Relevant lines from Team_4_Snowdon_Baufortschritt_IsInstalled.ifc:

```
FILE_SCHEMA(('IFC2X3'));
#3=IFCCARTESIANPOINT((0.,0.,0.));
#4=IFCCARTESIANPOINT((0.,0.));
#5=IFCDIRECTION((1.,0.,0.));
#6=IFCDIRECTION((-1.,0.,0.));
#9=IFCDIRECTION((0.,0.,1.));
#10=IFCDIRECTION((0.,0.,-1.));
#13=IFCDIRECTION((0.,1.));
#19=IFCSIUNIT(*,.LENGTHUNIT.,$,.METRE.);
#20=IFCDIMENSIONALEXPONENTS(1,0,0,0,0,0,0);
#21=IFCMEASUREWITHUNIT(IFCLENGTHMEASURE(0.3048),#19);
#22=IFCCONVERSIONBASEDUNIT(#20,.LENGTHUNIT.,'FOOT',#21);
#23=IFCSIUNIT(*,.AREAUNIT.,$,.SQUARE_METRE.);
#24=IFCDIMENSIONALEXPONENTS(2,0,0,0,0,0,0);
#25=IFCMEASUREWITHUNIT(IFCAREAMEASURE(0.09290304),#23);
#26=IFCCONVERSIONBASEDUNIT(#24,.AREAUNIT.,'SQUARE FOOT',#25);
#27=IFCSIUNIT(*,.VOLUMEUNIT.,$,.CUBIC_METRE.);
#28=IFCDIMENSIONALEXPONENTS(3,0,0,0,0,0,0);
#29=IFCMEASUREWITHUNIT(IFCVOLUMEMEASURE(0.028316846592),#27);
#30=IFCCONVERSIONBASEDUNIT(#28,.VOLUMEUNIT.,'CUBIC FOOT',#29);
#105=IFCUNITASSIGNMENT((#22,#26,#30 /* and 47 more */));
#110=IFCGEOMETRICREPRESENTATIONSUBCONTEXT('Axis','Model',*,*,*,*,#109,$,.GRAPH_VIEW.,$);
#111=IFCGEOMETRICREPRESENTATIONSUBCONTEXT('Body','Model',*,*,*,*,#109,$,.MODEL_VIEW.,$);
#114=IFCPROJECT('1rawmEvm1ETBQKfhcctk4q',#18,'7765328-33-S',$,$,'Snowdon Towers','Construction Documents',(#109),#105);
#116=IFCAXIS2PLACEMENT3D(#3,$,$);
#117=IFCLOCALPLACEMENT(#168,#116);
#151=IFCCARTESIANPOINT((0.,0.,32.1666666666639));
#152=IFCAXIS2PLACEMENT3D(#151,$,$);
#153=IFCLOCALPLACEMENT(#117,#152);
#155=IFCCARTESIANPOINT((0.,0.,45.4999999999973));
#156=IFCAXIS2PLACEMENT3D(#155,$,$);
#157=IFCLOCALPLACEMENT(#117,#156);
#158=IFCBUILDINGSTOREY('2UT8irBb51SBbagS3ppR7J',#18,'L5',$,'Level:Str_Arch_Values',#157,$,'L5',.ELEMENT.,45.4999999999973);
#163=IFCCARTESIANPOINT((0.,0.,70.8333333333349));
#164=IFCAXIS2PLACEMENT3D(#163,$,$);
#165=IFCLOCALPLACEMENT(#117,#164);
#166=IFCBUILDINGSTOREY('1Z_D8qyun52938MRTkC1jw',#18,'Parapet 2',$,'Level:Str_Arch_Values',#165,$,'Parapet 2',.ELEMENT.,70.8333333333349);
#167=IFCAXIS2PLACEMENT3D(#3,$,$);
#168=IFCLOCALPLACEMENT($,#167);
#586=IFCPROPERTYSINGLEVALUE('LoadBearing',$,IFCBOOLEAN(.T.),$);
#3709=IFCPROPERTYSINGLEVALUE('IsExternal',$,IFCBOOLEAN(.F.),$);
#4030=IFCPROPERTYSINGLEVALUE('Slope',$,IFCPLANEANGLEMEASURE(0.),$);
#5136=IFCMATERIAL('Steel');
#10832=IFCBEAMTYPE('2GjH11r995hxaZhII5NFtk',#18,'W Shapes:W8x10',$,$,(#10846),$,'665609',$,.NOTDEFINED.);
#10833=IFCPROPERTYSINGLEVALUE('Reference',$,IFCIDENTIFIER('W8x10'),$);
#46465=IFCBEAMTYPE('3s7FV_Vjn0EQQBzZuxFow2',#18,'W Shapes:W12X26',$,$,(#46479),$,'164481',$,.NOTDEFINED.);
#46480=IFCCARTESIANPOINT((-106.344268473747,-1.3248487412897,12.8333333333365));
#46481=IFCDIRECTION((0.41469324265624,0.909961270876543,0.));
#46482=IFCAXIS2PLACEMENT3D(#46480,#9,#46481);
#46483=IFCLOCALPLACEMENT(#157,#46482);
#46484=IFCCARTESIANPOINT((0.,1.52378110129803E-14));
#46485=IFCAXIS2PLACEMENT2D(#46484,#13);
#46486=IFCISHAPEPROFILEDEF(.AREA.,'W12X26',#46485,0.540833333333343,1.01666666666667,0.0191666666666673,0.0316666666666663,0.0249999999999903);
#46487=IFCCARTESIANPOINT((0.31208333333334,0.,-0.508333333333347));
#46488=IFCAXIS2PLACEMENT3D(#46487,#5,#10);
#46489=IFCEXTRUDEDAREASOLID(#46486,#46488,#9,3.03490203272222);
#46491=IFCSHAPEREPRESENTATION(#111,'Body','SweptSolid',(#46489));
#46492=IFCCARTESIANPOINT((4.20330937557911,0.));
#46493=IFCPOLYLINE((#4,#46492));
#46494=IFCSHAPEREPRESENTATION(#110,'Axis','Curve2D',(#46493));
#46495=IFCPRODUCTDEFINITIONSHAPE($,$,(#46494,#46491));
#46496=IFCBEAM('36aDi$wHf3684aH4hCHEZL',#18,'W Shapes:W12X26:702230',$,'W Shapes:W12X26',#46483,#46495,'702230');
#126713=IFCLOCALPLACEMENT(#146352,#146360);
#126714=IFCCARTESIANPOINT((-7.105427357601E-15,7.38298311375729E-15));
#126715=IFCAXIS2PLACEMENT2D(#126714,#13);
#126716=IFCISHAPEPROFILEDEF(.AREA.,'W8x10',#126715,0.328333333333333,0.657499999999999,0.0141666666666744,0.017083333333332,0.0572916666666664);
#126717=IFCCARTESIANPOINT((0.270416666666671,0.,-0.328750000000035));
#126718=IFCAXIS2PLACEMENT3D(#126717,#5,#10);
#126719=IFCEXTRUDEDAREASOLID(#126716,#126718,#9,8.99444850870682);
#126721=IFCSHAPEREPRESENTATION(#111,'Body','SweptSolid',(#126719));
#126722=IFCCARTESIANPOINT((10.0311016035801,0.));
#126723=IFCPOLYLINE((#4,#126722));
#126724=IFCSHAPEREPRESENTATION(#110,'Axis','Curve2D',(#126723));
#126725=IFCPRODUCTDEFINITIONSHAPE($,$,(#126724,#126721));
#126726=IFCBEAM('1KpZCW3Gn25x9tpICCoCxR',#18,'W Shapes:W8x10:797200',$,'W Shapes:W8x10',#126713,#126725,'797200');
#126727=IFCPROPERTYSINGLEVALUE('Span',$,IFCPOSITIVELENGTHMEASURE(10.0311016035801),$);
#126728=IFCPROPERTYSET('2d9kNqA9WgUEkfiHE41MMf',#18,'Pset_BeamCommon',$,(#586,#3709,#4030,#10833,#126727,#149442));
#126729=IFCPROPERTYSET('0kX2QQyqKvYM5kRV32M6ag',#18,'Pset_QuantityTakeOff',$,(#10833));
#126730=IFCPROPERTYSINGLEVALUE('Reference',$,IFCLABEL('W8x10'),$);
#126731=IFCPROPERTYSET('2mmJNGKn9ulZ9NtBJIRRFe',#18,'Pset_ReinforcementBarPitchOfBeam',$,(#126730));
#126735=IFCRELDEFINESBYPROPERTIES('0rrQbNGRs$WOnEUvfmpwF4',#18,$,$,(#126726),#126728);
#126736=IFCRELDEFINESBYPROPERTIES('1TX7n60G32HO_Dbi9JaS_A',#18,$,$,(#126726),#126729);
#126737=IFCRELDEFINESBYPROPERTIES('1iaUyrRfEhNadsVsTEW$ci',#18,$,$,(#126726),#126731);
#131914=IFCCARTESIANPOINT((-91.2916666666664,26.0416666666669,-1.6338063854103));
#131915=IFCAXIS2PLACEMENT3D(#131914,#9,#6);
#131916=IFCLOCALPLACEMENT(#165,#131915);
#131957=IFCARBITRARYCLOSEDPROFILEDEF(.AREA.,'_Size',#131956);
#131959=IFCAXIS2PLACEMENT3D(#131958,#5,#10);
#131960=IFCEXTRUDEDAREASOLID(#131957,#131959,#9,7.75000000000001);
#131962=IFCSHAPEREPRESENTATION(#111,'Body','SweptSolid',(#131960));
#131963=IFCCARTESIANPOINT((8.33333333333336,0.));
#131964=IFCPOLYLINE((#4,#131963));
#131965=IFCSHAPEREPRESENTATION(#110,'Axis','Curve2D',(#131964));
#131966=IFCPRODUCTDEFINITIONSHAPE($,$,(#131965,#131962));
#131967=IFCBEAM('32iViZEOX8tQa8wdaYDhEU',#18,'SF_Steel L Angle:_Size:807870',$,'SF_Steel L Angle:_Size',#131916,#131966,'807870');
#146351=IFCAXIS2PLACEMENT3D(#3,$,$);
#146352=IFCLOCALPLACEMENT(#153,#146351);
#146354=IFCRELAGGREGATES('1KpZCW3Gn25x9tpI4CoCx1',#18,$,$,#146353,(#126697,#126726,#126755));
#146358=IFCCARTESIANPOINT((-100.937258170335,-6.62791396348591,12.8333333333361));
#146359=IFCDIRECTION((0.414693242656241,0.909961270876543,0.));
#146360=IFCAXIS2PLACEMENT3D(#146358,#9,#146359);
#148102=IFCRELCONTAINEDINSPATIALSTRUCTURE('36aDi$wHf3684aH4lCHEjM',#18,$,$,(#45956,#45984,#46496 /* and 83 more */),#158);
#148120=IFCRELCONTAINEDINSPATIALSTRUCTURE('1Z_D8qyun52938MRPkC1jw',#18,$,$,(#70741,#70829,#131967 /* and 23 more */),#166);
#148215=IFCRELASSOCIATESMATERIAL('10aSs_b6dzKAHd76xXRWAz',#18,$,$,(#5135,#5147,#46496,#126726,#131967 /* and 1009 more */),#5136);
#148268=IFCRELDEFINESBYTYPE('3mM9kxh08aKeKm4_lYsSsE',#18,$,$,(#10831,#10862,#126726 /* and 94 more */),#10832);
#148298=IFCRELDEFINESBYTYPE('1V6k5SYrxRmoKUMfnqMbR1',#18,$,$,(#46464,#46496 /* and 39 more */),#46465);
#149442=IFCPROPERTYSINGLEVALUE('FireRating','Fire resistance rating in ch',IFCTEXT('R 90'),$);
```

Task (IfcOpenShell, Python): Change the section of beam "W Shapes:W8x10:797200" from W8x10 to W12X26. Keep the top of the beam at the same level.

```python
import ifcopenshell
import ifcopenshell.api.pset
import ifcopenshell.api.type
import ifcopenshell.util.element
import ifcopenshell.util.representation

model = ifcopenshell.open("Team_4_Snowdon_Baufortschritt_IsInstalled.ifc")

member = model.by_id(126726)
source = next(p for p in model.by_type("IfcIShapeProfileDef") if p.ProfileName == "W12X26")

body = ifcopenshell.util.representation.get_representation(member, "Model", "Body")
solid = body.Items[0]
old_profile = solid.SweptArea

# Copy the section's sizes but keep this member's own profile position.
profile = ifcopenshell.util.element.copy(model, source)
# Profiles are centred, so shift by half the change in depth to hold the top.
shift = (old_profile.OverallDepth - profile.OverallDepth) / 2
x, y = old_profile.Position.Location.Coordinates
up = (-1.0, 0.0)  # upwards, in the solid's own plane
location = model.createIfcCartesianPoint((x + up[0] * shift, y + up[1] * shift))
profile.Position = model.createIfcAxis2Placement2D(location, old_profile.Position.RefDirection)
solid.SweptArea = profile
if not model.get_total_inverses(old_profile):
    ifcopenshell.util.element.remove_deep2(model, old_profile)

new_type = model.by_guid("3s7FV_Vjn0EQQBzZuxFow2")
ifcopenshell.api.type.assign_type(
    model, related_objects=[member], relating_type=new_type, should_map_representations=False
)
member.Name = member.Name.replace("W8x10", "W12X26")
member.ObjectType = "W Shapes:W12X26"
pset = model.by_id(ifcopenshell.util.element.get_pset(member, "Pset_BeamCommon", should_inherit=False)["id"])
ifcopenshell.api.pset.edit_pset(model, pset=pset, properties={"Reference": "W12X26"})
pset = model.by_id(ifcopenshell.util.element.get_pset(member, "Pset_QuantityTakeOff", should_inherit=False)["id"])
ifcopenshell.api.pset.edit_pset(model, pset=pset, properties={"Reference": "W12X26"})
pset = model.by_id(ifcopenshell.util.element.get_pset(member, "Pset_ReinforcementBarPitchOfBeam", should_inherit=False)["id"])
ifcopenshell.api.pset.edit_pset(model, pset=pset, properties={"Reference": "W12X26"})

print(solid.SweptArea)

model.write("Team_4_Snowdon_Baufortschritt_IsInstalled_v2.ifc")
```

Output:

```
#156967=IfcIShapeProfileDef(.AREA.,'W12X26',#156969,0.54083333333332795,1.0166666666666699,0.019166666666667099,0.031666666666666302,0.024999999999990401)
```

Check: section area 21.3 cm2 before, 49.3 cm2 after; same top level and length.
